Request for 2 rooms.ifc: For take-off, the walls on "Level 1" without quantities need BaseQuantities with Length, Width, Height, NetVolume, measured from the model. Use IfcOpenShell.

First a look at what the model holds.

```python
import ifcopenshell
import ifcopenshell.util.element
import ifcopenshell.util.unit

model = ifcopenshell.open("2 rooms.ifc")
print(model.schema)
for unit_type in ("LENGTHUNIT", "AREAUNIT", "VOLUMEUNIT"):
    print(unit_type, ifcopenshell.util.unit.calculate_unit_scale(model, unit_type))
storey = next(s for s in model.by_type("IfcBuildingStorey") if s.Name == "Level 1")
walls = [e for e in ifcopenshell.util.element.get_decomposition(storey) if e.is_a("IfcWall")]
for e in sorted(walls, key=lambda e: e.id()):
    print(e.id(), e.is_a(), e.Name, list(ifcopenshell.util.element.get_psets(e, qtos_only=True)), sep=" | ")
```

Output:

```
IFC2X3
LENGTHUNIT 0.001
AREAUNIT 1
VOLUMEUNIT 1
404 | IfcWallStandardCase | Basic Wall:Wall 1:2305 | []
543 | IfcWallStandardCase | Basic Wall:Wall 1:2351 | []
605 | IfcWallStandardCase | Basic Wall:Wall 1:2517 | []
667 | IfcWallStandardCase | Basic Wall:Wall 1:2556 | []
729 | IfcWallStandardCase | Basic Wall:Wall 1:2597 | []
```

```python
import ifcopenshell
import ifcopenshell.api.pset
import ifcopenshell.geom
import ifcopenshell.util.element
import ifcopenshell.util.shape
import ifcopenshell.util.unit

model = ifcopenshell.open("2 rooms.ifc")
unit_scale = ifcopenshell.util.unit.calculate_unit_scale(model)
volume_scale = ifcopenshell.util.unit.calculate_unit_scale(model, "VOLUMEUNIT")
settings = ifcopenshell.geom.settings()

storey = next(s for s in model.by_type("IfcBuildingStorey") if s.Name == "Level 1")
walls = [e for e in ifcopenshell.util.element.get_decomposition(storey) if e.is_a("IfcWall")]

for e in sorted(walls, key=lambda e: e.id()):
    if ifcopenshell.util.element.get_psets(e, qtos_only=True, should_inherit=False):
        continue
    # Geometry comes back in metres, in the element's own axes.
    shape = ifcopenshell.geom.create_shape(settings, e)
    values = {
        "Length": ifcopenshell.util.shape.get_x(shape.geometry) / unit_scale,
        "Width": ifcopenshell.util.shape.get_y(shape.geometry) / unit_scale,
        "Height": ifcopenshell.util.shape.get_z(shape.geometry) / unit_scale,
        "NetVolume": ifcopenshell.util.shape.get_volume(shape.geometry) / volume_scale,
    }
    qto = ifcopenshell.api.pset.add_qto(model, product=e, name="BaseQuantities")
    ifcopenshell.api.pset.edit_qto(model, qto=qto, properties=values)
    print(e.id(), {k: round(v, 3) for k, v in values.items()})

model.write("2 rooms_edited.ifc")
```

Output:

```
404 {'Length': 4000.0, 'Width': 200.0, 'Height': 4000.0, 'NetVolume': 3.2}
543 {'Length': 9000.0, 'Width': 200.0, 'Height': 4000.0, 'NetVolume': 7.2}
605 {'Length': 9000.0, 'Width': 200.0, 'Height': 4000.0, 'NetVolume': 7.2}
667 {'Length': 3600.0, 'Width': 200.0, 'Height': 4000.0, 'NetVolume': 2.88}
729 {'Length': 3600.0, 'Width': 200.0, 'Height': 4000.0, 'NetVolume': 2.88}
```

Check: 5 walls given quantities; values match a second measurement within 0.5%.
